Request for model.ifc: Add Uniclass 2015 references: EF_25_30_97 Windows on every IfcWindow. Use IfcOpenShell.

First a look at what the model holds.

```python
import ifcopenshell

model = ifcopenshell.open("model.ifc")
print(model.schema)
print("classifications:", [c.Name for c in model.by_type("IfcClassification")])
for ifc_class in ("IfcDoor", "IfcRoof", "IfcStair", "IfcWall", "IfcWindow"):
    print(ifc_class, len(model.by_type(ifc_class)))
```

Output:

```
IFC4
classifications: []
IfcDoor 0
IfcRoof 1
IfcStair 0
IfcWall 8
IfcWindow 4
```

```python
import ifcopenshell
import ifcopenshell.api.classification

model = ifcopenshell.open("model.ifc")

system = ifcopenshell.api.classification.add_classification(model, classification="Uniclass 2015")

codes = {
    "IfcWindow": ("EF_25_30_97", "Windows"),
}
for ifc_class, (code, name) in codes.items():
    products = model.by_type(ifc_class)
    ifcopenshell.api.classification.add_reference(
        model, products=products, classification=system, identification=code, name=name
    )
    print(code, len(products))

model.write("model_rev.ifc")
```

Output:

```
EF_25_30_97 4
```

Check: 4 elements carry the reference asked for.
